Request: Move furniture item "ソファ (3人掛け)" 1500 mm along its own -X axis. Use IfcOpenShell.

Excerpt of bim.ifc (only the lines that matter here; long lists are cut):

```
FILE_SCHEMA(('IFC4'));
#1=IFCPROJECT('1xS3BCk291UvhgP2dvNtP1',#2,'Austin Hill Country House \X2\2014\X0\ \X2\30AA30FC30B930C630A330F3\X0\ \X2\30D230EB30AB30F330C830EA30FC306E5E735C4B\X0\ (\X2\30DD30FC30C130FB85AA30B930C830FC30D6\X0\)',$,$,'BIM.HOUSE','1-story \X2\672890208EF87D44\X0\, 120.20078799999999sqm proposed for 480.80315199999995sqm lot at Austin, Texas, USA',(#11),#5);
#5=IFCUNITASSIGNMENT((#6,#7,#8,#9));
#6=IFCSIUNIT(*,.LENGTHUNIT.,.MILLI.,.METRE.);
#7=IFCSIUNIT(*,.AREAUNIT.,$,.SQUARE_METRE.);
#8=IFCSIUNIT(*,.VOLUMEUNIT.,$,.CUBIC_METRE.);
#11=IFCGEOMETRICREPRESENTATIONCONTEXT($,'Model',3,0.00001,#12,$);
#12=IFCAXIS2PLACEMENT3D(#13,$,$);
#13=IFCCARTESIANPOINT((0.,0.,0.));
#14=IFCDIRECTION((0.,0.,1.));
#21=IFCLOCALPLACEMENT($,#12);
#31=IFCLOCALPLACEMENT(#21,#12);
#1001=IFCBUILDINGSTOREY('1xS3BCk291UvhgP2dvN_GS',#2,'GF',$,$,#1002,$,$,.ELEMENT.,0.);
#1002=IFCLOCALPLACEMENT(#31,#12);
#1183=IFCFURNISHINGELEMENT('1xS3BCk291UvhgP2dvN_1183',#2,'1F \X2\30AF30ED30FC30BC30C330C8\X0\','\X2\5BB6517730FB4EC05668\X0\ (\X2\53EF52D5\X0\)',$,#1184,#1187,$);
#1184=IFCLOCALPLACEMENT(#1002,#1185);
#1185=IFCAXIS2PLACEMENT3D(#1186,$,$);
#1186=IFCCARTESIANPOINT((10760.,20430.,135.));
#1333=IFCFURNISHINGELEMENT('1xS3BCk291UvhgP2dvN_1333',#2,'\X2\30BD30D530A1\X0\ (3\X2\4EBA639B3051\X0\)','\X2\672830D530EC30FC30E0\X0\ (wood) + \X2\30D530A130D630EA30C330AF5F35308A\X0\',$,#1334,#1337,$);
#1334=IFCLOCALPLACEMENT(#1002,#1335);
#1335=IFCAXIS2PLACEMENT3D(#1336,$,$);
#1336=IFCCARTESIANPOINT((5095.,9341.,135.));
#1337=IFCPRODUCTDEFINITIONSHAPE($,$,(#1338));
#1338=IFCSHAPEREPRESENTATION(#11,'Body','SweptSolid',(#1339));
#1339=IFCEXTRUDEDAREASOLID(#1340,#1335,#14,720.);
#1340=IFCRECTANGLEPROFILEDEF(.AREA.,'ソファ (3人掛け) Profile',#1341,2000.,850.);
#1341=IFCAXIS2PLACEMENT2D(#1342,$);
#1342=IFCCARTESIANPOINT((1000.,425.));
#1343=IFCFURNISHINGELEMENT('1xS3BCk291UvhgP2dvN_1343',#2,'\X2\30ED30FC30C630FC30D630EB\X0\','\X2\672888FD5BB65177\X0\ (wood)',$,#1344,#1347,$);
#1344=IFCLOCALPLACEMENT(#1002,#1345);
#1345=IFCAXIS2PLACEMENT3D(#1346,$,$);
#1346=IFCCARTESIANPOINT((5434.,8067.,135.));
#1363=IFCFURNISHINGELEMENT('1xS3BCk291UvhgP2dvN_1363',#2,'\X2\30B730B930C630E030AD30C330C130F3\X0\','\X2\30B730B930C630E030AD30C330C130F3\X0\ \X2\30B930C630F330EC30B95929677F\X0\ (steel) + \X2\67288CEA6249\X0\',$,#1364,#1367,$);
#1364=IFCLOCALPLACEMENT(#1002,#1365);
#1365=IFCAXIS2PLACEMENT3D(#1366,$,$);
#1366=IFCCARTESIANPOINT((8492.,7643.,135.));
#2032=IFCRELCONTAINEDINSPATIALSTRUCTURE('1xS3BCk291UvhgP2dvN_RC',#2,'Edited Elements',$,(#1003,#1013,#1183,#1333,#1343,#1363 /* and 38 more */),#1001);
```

```python
import ifcopenshell
import ifcopenshell.api.geometry
import ifcopenshell.util.placement
import ifcopenshell.util.unit

model = ifcopenshell.open("bim.ifc")
unit_scale = ifcopenshell.util.unit.calculate_unit_scale(model)

item = model.by_guid("1xS3BCk291UvhgP2dvN_1333")
matrix = ifcopenshell.util.placement.get_local_placement(item.ObjectPlacement)
matrix[:3, 3] -= matrix[:3, 0] * 1.5 / unit_scale
ifcopenshell.api.geometry.edit_object_placement(model, product=item, matrix=matrix, is_si=False)

print(ifcopenshell.util.placement.get_local_placement(item.ObjectPlacement).round(3) + 0.0)

model.write("bim_edited.ifc")
```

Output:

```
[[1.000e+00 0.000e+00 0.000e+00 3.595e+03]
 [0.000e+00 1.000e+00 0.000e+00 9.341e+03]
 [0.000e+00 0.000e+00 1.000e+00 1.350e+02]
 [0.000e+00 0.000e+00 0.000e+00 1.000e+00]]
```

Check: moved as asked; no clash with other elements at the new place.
